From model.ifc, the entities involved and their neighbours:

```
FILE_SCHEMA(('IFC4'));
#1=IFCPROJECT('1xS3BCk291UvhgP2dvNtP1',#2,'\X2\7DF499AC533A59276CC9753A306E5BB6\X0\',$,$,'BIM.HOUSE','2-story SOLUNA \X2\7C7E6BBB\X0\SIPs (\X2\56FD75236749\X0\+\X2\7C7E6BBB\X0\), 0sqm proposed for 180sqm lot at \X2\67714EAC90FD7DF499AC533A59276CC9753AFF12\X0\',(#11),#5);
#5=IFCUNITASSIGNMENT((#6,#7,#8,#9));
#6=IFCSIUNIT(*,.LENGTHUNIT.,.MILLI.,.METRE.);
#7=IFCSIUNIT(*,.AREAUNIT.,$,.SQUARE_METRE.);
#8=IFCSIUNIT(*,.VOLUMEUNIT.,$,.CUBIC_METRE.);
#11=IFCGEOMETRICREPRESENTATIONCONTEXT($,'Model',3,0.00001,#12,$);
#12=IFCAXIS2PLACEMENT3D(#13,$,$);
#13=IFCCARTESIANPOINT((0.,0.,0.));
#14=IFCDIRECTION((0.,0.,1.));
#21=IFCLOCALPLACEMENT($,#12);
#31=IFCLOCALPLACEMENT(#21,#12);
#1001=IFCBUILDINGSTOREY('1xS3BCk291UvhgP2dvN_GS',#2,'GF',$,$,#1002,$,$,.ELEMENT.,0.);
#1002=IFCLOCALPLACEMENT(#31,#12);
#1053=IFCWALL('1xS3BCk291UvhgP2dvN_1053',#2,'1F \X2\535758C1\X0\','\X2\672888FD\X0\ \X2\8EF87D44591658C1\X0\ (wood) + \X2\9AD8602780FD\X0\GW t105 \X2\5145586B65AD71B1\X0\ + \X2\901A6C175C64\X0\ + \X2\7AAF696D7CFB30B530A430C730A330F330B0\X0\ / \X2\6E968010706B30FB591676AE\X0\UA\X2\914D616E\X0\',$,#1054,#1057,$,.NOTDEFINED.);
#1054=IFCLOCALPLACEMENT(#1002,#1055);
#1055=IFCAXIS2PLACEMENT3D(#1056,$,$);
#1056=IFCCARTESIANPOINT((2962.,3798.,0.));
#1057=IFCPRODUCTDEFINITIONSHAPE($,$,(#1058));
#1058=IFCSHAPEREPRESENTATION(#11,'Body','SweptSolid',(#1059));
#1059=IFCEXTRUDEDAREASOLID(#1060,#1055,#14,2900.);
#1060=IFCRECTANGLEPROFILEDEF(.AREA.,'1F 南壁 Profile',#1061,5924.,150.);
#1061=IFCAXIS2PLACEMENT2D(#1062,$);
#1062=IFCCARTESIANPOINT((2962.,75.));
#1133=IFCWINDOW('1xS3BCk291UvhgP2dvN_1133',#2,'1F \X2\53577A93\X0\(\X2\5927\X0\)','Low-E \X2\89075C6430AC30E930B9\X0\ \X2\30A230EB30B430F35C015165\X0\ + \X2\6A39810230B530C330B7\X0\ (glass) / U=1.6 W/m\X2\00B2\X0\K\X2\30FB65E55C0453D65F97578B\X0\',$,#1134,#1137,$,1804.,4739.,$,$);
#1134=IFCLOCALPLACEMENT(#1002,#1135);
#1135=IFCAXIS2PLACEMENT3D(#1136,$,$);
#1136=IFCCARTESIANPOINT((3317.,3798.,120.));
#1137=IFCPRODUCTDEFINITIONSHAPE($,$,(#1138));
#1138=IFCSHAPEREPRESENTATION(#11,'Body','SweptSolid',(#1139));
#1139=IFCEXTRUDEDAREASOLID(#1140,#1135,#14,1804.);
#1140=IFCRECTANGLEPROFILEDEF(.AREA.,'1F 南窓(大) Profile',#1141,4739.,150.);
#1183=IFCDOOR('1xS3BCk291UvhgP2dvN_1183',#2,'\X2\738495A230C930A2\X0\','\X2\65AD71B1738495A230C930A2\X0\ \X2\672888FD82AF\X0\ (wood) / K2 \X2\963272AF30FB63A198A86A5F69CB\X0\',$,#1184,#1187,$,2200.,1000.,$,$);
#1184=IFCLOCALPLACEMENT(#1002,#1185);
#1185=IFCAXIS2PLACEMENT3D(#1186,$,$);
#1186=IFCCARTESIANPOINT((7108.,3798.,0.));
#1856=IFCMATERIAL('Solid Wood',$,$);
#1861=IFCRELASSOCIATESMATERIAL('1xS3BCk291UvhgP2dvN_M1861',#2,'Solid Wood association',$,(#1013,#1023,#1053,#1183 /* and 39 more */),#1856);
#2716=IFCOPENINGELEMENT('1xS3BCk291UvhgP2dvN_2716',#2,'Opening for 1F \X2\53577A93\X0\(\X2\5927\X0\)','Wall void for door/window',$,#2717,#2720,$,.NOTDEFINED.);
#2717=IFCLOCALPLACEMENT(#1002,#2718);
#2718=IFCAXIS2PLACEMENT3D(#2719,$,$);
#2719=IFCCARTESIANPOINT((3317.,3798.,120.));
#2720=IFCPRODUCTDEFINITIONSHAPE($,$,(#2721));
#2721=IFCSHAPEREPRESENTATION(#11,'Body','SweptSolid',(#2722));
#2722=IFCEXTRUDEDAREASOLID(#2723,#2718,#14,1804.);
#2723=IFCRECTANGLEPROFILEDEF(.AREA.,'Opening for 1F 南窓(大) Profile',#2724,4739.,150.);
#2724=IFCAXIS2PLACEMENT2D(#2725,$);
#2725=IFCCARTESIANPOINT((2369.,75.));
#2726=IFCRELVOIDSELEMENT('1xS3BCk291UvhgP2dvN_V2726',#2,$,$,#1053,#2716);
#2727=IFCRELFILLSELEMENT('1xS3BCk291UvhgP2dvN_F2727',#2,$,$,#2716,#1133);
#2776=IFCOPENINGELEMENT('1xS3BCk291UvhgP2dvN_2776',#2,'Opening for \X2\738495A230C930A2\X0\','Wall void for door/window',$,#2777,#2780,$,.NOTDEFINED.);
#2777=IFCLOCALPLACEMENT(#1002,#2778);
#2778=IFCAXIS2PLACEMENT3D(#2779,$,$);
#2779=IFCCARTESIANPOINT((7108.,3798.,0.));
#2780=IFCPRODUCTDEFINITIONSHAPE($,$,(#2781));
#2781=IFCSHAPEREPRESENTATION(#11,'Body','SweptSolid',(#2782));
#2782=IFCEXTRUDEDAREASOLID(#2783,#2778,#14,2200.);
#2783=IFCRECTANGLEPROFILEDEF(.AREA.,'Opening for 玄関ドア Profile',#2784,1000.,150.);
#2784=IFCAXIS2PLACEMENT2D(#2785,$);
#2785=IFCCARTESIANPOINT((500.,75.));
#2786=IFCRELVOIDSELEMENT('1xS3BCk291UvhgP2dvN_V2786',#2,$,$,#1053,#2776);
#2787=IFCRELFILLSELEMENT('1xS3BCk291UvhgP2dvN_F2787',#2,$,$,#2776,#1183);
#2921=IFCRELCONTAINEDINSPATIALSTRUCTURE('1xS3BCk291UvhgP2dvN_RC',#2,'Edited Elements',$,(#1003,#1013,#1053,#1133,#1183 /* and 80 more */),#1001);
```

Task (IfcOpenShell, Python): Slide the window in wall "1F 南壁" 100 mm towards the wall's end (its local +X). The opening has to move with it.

```python
import ifcopenshell
import ifcopenshell.api.geometry
import ifcopenshell.util.placement
import ifcopenshell.util.unit

model = ifcopenshell.open("model.ifc")
unit_scale = ifcopenshell.util.unit.calculate_unit_scale(model)

window = model.by_guid("1xS3BCk291UvhgP2dvN_1133")
opening = window.FillsVoids[0].RelatingOpeningElement
wall = opening.VoidsElements[0].RelatingBuildingElement

wall_matrix = ifcopenshell.util.placement.get_local_placement(wall.ObjectPlacement)
shift = wall_matrix[:3, 0] * 0.1 / unit_scale
before = ifcopenshell.util.placement.get_local_placement(window.ObjectPlacement)[:3, 3].copy()

# The window is not placed relative to its opening, so move both.
for product in (opening, window):
    matrix = ifcopenshell.util.placement.get_local_placement(product.ObjectPlacement)
    matrix[:3, 3] += shift
    ifcopenshell.api.geometry.edit_object_placement(model, product=product, matrix=matrix, is_si=False)

after = ifcopenshell.util.placement.get_local_placement(window.ObjectPlacement)[:3, 3]
print("window moved by", (after - before).round(3) + 0.0)

model.write("model-out.ifc")
```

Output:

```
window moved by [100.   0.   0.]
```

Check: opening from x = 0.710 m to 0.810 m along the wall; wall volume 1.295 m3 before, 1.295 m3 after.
